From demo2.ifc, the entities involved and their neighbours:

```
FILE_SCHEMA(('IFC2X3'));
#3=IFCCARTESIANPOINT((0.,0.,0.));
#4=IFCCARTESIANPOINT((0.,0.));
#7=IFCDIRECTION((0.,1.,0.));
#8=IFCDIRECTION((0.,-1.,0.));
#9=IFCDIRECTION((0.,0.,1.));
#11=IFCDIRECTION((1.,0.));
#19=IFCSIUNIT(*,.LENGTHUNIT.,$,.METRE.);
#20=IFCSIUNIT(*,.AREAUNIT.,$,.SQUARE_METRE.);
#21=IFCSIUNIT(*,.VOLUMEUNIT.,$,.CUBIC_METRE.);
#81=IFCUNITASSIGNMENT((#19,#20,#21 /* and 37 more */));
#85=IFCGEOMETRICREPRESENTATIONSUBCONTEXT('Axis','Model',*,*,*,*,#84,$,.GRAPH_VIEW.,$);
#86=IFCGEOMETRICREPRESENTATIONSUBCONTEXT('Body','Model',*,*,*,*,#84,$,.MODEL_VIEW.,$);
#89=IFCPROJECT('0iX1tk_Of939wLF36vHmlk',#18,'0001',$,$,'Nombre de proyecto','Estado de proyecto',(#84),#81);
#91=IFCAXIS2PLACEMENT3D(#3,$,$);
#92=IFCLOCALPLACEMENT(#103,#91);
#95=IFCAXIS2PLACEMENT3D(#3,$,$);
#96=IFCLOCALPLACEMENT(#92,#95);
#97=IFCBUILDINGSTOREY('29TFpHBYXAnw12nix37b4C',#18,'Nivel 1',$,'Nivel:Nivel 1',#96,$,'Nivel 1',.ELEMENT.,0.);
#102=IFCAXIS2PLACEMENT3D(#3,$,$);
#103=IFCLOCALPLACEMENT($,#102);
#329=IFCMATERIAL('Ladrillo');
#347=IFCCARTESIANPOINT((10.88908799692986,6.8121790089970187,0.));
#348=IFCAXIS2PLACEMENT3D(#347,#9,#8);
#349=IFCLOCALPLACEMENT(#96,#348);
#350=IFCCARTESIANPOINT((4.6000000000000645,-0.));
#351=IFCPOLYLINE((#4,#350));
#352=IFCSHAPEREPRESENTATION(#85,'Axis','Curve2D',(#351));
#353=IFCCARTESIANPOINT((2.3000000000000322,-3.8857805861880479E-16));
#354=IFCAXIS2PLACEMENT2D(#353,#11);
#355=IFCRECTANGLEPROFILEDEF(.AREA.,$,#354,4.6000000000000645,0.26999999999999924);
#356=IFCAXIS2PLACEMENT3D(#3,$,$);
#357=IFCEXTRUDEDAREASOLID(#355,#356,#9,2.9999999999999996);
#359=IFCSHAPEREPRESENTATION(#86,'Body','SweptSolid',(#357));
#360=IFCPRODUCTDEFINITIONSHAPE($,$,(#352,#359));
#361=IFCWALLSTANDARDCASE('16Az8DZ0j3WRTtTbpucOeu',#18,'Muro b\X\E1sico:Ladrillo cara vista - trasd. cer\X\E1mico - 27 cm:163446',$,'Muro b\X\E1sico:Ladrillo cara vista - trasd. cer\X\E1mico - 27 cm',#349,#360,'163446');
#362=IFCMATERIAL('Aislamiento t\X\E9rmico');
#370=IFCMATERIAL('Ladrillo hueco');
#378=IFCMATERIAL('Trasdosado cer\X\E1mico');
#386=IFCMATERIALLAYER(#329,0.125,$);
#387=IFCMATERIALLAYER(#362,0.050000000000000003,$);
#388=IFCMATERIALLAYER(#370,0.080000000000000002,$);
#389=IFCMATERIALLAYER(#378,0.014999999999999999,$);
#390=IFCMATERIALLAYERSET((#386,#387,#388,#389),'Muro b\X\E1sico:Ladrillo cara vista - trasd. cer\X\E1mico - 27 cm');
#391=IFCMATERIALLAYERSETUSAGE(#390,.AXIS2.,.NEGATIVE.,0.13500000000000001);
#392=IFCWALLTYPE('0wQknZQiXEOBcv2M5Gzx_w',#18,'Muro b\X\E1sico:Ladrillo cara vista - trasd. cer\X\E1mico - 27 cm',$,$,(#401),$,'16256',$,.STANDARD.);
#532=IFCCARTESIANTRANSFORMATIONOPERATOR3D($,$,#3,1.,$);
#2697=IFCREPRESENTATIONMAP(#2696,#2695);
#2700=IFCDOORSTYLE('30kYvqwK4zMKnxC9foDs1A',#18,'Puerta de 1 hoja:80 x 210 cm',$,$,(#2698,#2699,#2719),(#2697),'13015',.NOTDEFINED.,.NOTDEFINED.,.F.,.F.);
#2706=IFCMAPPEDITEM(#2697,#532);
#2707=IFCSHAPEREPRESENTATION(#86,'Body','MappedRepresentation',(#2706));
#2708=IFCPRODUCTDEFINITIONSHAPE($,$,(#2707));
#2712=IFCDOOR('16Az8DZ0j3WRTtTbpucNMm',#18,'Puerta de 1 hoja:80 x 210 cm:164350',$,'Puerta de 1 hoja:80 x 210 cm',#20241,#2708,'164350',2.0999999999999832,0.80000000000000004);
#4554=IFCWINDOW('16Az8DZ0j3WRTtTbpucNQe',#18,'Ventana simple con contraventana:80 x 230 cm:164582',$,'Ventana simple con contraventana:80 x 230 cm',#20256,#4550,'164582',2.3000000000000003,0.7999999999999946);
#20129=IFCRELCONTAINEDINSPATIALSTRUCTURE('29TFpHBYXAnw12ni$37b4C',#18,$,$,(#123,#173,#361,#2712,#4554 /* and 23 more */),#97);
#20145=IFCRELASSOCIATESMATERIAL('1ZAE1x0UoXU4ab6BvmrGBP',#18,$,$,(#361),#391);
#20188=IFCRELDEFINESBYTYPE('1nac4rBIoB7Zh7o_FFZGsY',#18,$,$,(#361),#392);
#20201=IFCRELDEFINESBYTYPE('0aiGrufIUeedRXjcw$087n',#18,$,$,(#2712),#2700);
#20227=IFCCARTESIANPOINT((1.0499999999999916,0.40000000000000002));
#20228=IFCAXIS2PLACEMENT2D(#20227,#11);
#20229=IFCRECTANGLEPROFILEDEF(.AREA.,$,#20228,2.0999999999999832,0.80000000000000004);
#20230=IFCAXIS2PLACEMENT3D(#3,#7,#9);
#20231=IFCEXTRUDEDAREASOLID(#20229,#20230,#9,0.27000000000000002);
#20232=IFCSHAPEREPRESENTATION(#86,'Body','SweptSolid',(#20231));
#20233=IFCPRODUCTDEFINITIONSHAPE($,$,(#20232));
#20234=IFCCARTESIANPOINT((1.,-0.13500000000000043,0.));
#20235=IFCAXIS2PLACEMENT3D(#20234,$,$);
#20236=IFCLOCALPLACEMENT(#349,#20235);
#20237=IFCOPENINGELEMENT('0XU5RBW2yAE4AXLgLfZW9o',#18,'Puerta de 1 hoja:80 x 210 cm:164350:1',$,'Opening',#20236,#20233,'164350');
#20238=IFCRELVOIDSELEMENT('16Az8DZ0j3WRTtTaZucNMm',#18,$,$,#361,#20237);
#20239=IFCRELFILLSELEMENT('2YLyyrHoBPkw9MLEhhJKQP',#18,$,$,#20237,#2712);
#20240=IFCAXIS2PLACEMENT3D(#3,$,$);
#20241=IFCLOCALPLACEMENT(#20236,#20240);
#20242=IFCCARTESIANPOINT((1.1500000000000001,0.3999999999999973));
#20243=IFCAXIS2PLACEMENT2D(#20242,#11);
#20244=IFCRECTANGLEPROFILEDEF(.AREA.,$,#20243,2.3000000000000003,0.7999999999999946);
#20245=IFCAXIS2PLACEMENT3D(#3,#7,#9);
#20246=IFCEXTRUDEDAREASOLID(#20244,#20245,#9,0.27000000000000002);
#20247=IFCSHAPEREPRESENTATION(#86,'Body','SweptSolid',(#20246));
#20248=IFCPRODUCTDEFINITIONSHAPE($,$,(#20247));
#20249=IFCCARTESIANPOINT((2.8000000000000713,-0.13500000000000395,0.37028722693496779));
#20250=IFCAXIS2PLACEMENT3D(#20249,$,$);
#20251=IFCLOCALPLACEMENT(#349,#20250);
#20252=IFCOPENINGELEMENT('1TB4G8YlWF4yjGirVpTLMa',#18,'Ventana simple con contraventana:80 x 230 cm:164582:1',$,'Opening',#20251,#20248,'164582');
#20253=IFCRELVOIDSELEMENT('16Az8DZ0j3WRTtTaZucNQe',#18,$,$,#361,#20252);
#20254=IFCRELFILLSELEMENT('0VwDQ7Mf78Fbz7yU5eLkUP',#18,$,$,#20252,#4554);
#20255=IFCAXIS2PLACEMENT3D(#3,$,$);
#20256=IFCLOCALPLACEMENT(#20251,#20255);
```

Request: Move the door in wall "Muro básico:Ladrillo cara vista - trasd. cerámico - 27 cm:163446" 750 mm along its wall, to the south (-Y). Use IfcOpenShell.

```python
import ifcopenshell
import ifcopenshell.api.geometry
import ifcopenshell.util.placement
import ifcopenshell.util.unit

model = ifcopenshell.open("demo2.ifc")
unit_scale = ifcopenshell.util.unit.calculate_unit_scale(model)

door = model.by_guid("16Az8DZ0j3WRTtTbpucNMm")
opening = door.FillsVoids[0].RelatingOpeningElement
wall = opening.VoidsElements[0].RelatingBuildingElement

wall_matrix = ifcopenshell.util.placement.get_local_placement(wall.ObjectPlacement)
shift = wall_matrix[:3, 0] * 0.75 / unit_scale
before = ifcopenshell.util.placement.get_local_placement(door.ObjectPlacement)[:3, 3].copy()

# The door is placed relative to its opening, so it follows when the opening moves.
matrix = ifcopenshell.util.placement.get_local_placement(opening.ObjectPlacement)
matrix[:3, 3] += shift
ifcopenshell.api.geometry.edit_object_placement(
    model, product=opening, matrix=matrix, is_si=False, should_transform_children=True
)

after = ifcopenshell.util.placement.get_local_placement(door.ObjectPlacement)[:3, 3]
print("door moved by", (after - before).round(3) + 0.0)

model.write("demo2_rev.ifc")
```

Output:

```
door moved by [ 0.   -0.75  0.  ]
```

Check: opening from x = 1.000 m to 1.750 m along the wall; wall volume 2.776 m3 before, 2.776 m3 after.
